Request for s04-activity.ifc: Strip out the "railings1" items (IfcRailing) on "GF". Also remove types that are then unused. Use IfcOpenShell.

First a look at what the model holds.

```python
import ifcopenshell
import ifcopenshell.util.element

model = ifcopenshell.open("s04-activity.ifc")
print(model.schema)
storey = next(s for s in model.by_type("IfcBuildingStorey") if s.Name == "GF")
railings = [e for e in ifcopenshell.util.element.get_decomposition(storey) if e.is_a("IfcRailing")]
seen = {}
for e in railings:
    element_type = ifcopenshell.util.element.get_type(e)
    name = element_type.Name if element_type not in (None, e) else None
    seen[name] = seen.get(name, 0) + 1
for name, count in sorted(seen.items(), key=str):
    print(count, "x", name)
```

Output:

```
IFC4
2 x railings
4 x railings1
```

```python
import ifcopenshell
import ifcopenshell.api.root
import ifcopenshell.util.element

model = ifcopenshell.open("s04-activity.ifc")

storey = next(s for s in model.by_type("IfcBuildingStorey") if s.Name == "GF")
railings = [e for e in ifcopenshell.util.element.get_decomposition(storey) if e.is_a("IfcRailing")]
targets = [e for e in railings if (t := ifcopenshell.util.element.get_type(e)) not in (None, e) and t.Name == "railings1"]
types = {ifcopenshell.util.element.get_type(e) for e in targets} - {None, *targets}

for e in targets:
    ifcopenshell.api.root.remove_product(model, product=e)
print(len(targets), "removed")

unused = [t for t in types if not ifcopenshell.util.element.get_types(t)]
for t in unused:
    ifcopenshell.api.root.remove_product(model, product=t)
print(len(unused), "unused types removed")

model.write("s04-activity_rev.ifc")
```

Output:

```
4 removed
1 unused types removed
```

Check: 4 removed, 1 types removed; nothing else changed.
